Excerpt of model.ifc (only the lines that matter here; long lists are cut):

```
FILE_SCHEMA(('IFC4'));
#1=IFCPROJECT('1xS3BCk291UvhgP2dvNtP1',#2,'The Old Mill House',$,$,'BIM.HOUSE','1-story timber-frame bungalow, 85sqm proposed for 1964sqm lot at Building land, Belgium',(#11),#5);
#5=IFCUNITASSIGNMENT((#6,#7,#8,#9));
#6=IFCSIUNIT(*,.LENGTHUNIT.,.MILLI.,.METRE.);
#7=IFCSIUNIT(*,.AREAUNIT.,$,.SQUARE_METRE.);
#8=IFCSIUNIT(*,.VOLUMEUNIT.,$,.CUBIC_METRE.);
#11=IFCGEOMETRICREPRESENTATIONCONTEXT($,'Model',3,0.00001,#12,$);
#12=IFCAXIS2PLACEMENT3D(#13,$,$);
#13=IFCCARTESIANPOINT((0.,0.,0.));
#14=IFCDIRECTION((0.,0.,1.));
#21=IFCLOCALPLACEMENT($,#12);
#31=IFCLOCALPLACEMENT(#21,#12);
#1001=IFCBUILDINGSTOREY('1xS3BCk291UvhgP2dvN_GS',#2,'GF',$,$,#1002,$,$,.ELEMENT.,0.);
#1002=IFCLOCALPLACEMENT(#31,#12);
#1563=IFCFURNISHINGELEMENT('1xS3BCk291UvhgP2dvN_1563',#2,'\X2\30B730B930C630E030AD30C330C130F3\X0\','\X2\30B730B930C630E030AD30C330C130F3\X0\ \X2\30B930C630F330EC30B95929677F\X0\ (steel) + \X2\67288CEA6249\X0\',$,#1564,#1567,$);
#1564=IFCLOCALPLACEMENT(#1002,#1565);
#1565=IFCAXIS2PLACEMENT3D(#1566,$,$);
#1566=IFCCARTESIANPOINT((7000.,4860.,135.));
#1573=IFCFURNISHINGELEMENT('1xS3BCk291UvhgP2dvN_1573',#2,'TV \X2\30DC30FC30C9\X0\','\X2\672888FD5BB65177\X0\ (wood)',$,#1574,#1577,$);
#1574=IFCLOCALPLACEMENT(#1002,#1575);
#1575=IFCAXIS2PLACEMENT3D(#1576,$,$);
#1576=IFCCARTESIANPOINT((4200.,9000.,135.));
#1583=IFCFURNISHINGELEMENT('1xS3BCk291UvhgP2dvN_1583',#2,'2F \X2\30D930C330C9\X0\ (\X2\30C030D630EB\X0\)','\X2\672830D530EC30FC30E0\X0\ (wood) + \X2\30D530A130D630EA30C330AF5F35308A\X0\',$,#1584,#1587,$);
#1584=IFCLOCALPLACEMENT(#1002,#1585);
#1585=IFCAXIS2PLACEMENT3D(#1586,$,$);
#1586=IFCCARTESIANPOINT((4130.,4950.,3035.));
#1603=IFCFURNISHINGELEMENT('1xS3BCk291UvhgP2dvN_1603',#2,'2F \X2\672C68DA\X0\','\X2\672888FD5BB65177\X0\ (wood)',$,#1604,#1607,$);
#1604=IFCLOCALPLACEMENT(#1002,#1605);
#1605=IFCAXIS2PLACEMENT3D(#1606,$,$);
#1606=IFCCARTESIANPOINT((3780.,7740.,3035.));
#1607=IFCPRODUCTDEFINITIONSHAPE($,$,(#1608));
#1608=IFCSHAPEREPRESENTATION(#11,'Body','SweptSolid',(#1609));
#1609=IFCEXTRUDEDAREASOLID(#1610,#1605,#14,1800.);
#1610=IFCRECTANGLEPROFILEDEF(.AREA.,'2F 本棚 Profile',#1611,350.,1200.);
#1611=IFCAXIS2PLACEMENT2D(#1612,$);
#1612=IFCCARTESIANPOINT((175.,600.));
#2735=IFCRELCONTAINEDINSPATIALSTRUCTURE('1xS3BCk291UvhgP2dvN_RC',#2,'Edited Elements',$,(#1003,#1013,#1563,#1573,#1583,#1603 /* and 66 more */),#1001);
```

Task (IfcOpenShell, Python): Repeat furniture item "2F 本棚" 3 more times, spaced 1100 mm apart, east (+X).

```python
import numpy as np
import ifcopenshell
import ifcopenshell.api.geometry
import ifcopenshell.api.root
import ifcopenshell.util.element
import ifcopenshell.util.placement

model = ifcopenshell.open("model.ifc")


def reuse_history(source, copy):
    """copy_class also copies each property set's owner history, people and application; keep the originals."""
    for rel in copy.IsDefinedBy:
        if rel.is_a("IfcRelDefinesByProperties") and (history := rel.RelatingPropertyDefinition.OwnerHistory):
            rel.RelatingPropertyDefinition.OwnerHistory = source.OwnerHistory
            ifcopenshell.util.element.remove_deep2(model, history)


source = model.by_guid("1xS3BCk291UvhgP2dvN_1603")
base = ifcopenshell.util.placement.get_local_placement(source.ObjectPlacement)
step = np.array([1.0, 0.0, 0.0]) * 1100.0

for i in range(1, 4):
    copy = ifcopenshell.api.root.copy_class(model, product=source)
    copy.Representation = ifcopenshell.util.element.copy_deep(
        model, source.Representation, exclude=["IfcGeometricRepresentationContext", "IfcRepresentationMap"]
    )
    reuse_history(source, copy)
    matrix = base.copy()
    matrix[:3, 3] += i * step
    print("added at", matrix[:3, 3].round(3) + 0.0)
    ifcopenshell.api.geometry.edit_object_placement(model, product=copy, matrix=matrix, is_si=False)

model.write("model_rev.ifc")
```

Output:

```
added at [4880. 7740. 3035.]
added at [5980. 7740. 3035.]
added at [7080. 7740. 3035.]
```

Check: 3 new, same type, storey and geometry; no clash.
